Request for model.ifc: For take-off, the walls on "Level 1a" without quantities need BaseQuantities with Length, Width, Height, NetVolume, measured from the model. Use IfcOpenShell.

First a look at what the model holds.

```python
import ifcopenshell
import ifcopenshell.util.element
import ifcopenshell.util.unit

model = ifcopenshell.open("model.ifc")
print(model.schema)
for unit_type in ("LENGTHUNIT", "AREAUNIT", "VOLUMEUNIT"):
    print(unit_type, ifcopenshell.util.unit.calculate_unit_scale(model, unit_type))
storey = next(s for s in model.by_type("IfcBuildingStorey") if s.Name == "Level 1a")
walls = [e for e in ifcopenshell.util.element.get_decomposition(storey) if e.is_a("IfcWall")]
for e in sorted(walls, key=lambda e: e.id()):
    print(e.id(), e.is_a(), e.Name, list(ifcopenshell.util.element.get_psets(e, qtos_only=True)), sep=" | ")
```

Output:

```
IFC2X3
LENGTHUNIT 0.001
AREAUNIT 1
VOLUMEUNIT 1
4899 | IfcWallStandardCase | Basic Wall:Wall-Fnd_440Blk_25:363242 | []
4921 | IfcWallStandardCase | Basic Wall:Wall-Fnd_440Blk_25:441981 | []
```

```python
import ifcopenshell
import ifcopenshell.api.pset
import ifcopenshell.geom
import ifcopenshell.util.element
import ifcopenshell.util.shape
import ifcopenshell.util.unit

model = ifcopenshell.open("model.ifc")
unit_scale = ifcopenshell.util.unit.calculate_unit_scale(model)
volume_scale = ifcopenshell.util.unit.calculate_unit_scale(model, "VOLUMEUNIT")
settings = ifcopenshell.geom.settings()

storey = next(s for s in model.by_type("IfcBuildingStorey") if s.Name == "Level 1a")
walls = [e for e in ifcopenshell.util.element.get_decomposition(storey) if e.is_a("IfcWall")]

for e in sorted(walls, key=lambda e: e.id()):
    if ifcopenshell.util.element.get_psets(e, qtos_only=True, should_inherit=False):
        continue
    # Geometry comes back in metres, in the element's own axes.
    shape = ifcopenshell.geom.create_shape(settings, e)
    values = {
        "Length": ifcopenshell.util.shape.get_x(shape.geometry) / unit_scale,
        "Width": ifcopenshell.util.shape.get_y(shape.geometry) / unit_scale,
        "Height": ifcopenshell.util.shape.get_z(shape.geometry) / unit_scale,
        "NetVolume": ifcopenshell.util.shape.get_volume(shape.geometry) / volume_scale,
    }
    qto = ifcopenshell.api.pset.add_qto(model, product=e, name="BaseQuantities")
    ifcopenshell.api.pset.edit_qto(model, qto=qto, properties=values)
    print(e.id(), {k: round(v, 3) for k, v in values.items()})

model.write("model_rev.ifc")
```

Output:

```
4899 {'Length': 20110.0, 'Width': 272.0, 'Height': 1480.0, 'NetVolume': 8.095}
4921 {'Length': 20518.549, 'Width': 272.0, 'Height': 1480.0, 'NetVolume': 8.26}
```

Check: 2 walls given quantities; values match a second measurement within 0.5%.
